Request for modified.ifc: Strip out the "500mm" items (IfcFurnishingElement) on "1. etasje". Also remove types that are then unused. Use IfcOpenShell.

First a look at what the model holds.

```python
import ifcopenshell
import ifcopenshell.util.element

model = ifcopenshell.open("modified.ifc")
print(model.schema)
storey = next(s for s in model.by_type("IfcBuildingStorey") if s.Name == "1. etasje")
furniture = [e for e in ifcopenshell.util.element.get_decomposition(storey) if e.is_a("IfcFurnishingElement")]
seen = {}
for e in furniture:
    element_type = ifcopenshell.util.element.get_type(e)
    name = element_type.Name if element_type not in (None, e) else None
    seen[name] = seen.get(name, 0) + 1
for name, count in sorted(seen.items(), key=str):
    print(count, "x", name)
```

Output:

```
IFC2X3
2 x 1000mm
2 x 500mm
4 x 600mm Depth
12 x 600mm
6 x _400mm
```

```python
import ifcopenshell
import ifcopenshell.api.root
import ifcopenshell.util.element

model = ifcopenshell.open("modified.ifc")

storey = next(s for s in model.by_type("IfcBuildingStorey") if s.Name == "1. etasje")
furniture = [e for e in ifcopenshell.util.element.get_decomposition(storey) if e.is_a("IfcFurnishingElement")]
targets = [e for e in furniture if (t := ifcopenshell.util.element.get_type(e)) not in (None, e) and t.Name == "500mm"]
types = {ifcopenshell.util.element.get_type(e) for e in targets} - {None, *targets}

for e in targets:
    ifcopenshell.api.root.remove_product(model, product=e)
print(len(targets), "removed")

unused = [t for t in types if not ifcopenshell.util.element.get_types(t)]
for t in unused:
    ifcopenshell.api.root.remove_product(model, product=t)
print(len(unused), "unused types removed")

model.write("modified_rev.ifc")
```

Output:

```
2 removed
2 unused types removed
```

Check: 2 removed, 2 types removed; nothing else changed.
